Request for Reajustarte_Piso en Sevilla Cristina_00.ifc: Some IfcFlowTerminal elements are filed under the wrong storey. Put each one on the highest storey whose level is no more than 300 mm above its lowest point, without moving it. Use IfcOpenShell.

First a look at what the model holds.

```python
import ifcopenshell
import ifcopenshell.util.element
import ifcopenshell.util.placement

model = ifcopenshell.open("Reajustarte_Piso en Sevilla Cristina_00.ifc")
print(model.schema)
for storey in model.by_type("IfcBuildingStorey"):
    level = ifcopenshell.util.placement.get_storey_elevation(storey)
    count = sum(e.is_a("IfcFlowTerminal") for e in ifcopenshell.util.element.get_contained(storey))
    print(storey.id(), storey.Name, round(level, 3), count, sep=" | ")
```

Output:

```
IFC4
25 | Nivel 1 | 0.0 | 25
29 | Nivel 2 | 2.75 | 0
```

```python
import ifcopenshell
import ifcopenshell.api.spatial
import ifcopenshell.geom
import ifcopenshell.util.element
import ifcopenshell.util.placement
import ifcopenshell.util.shape
import ifcopenshell.util.unit

model = ifcopenshell.open("Reajustarte_Piso en Sevilla Cristina_00.ifc")
unit_scale = ifcopenshell.util.unit.calculate_unit_scale(model)
settings = ifcopenshell.geom.settings()

levels = sorted(
    ((ifcopenshell.util.placement.get_storey_elevation(s) * unit_scale, s) for s in model.by_type("IfcBuildingStorey")),
    key=lambda pair: pair[0],
)

for e in model.by_type("IfcFlowTerminal"):
    current = e.ContainedInStructure[0].RelatingStructure if e.ContainedInStructure else None
    if current is None or not current.is_a("IfcBuildingStorey"):
        continue
    shape = ifcopenshell.geom.create_shape(settings, e)
    bottom = ifcopenshell.util.shape.get_shape_bottom_elevation(shape, shape.geometry)
    below = [s for level, s in levels if level <= bottom + 0.3]
    storey = below[-1] if below else levels[0][1]
    if storey != current:
        # assign_container keeps the world position.
        ifcopenshell.api.spatial.assign_container(model, products=[e], relating_structure=storey)
        print(e.id(), current.Name, "->", storey.Name)

model.write("Reajustarte_Piso en Sevilla Cristina_00_v2.ifc")
```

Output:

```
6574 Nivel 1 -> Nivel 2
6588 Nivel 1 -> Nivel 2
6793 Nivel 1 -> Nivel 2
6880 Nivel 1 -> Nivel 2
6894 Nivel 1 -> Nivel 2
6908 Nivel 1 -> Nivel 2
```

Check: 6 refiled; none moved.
